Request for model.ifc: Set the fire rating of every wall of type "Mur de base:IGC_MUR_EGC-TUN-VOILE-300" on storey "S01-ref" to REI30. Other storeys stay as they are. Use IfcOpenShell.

First a look at what the model holds.

```python
import ifcopenshell
import ifcopenshell.util.element

model = ifcopenshell.open("model.ifc")
print(model.schema)
storey = next(s for s in model.by_type("IfcBuildingStorey") if s.Name == "S01-ref")
walls = [e for e in ifcopenshell.util.element.get_decomposition(storey) if e.is_a("IfcWall")]
seen = {}
for e in walls:
    element_type = ifcopenshell.util.element.get_type(e)
    key = (element_type.Name if element_type != e and element_type else None, ifcopenshell.util.element.get_pset(e, "Pset_WallCommon", "FireRating"))
    seen[key] = seen.get(key, 0) + 1
for (name, value), count in sorted(seen.items(), key=str):
    print(count, "x", name, "|", value)
```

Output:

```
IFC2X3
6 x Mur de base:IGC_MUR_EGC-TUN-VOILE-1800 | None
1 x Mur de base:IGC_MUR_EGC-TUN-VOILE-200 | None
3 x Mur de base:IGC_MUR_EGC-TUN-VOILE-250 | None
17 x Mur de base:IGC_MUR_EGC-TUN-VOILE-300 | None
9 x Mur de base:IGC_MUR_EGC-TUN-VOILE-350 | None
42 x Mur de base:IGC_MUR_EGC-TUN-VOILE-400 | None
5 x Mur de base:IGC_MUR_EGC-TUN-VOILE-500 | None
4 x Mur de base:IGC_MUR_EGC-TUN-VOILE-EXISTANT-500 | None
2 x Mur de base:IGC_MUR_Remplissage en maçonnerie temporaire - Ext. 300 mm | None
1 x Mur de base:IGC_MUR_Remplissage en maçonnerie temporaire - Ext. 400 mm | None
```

```python
import ifcopenshell
import ifcopenshell.api.pset
import ifcopenshell.util.element

model = ifcopenshell.open("model.ifc")

storey = next(s for s in model.by_type("IfcBuildingStorey") if s.Name == "S01-ref")
walls = [e for e in ifcopenshell.util.element.get_decomposition(storey) if e.is_a("IfcWall")]

count = 0
for e in walls:
    element_type = ifcopenshell.util.element.get_type(e)
    if element_type in (None, e) or element_type.Name != "Mur de base:IGC_MUR_EGC-TUN-VOILE-300":
        continue
    # add_pset returns the element's existing set when there is one.
    pset = ifcopenshell.api.pset.add_pset(model, product=e, name="Pset_WallCommon")
    ifcopenshell.api.pset.edit_pset(model, pset=pset, properties={"FireRating": "REI30"})
    count += 1

print(count, "walls updated")

model.write("model_v2.ifc")
```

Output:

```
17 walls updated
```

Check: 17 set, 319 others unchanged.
